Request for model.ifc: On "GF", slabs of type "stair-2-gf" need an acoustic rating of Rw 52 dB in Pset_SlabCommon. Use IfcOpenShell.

First a look at what the model holds.

```python
import ifcopenshell
import ifcopenshell.util.element

model = ifcopenshell.open("model.ifc")
print(model.schema)
storey = next(s for s in model.by_type("IfcBuildingStorey") if s.Name == "GF")
slabs = [e for e in ifcopenshell.util.element.get_decomposition(storey) if e.is_a("IfcSlab")]
seen = {}
for e in slabs:
    element_type = ifcopenshell.util.element.get_type(e)
    key = (element_type.Name if element_type != e and element_type else None, ifcopenshell.util.element.get_pset(e, "Pset_SlabCommon", "AcousticRating"))
    seen[key] = seen.get(key, 0) + 1
for (name, value), count in sorted(seen.items(), key=str):
    print(count, "x", name, "|", value)
```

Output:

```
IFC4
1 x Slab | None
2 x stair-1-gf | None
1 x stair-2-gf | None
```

```python
import ifcopenshell
import ifcopenshell.api.pset
import ifcopenshell.util.element

model = ifcopenshell.open("model.ifc")

storey = next(s for s in model.by_type("IfcBuildingStorey") if s.Name == "GF")
slabs = [e for e in ifcopenshell.util.element.get_decomposition(storey) if e.is_a("IfcSlab")]

count = 0
for e in slabs:
    element_type = ifcopenshell.util.element.get_type(e)
    if element_type in (None, e) or element_type.Name != "stair-2-gf":
        continue
    # add_pset returns the element's existing set when there is one.
    pset = ifcopenshell.api.pset.add_pset(model, product=e, name="Pset_SlabCommon")
    ifcopenshell.api.pset.edit_pset(model, pset=pset, properties={"AcousticRating": "Rw 52 dB"})
    count += 1

print(count, "slabs updated")

model.write("model_rev.ifc")
```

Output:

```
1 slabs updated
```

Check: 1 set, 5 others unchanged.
